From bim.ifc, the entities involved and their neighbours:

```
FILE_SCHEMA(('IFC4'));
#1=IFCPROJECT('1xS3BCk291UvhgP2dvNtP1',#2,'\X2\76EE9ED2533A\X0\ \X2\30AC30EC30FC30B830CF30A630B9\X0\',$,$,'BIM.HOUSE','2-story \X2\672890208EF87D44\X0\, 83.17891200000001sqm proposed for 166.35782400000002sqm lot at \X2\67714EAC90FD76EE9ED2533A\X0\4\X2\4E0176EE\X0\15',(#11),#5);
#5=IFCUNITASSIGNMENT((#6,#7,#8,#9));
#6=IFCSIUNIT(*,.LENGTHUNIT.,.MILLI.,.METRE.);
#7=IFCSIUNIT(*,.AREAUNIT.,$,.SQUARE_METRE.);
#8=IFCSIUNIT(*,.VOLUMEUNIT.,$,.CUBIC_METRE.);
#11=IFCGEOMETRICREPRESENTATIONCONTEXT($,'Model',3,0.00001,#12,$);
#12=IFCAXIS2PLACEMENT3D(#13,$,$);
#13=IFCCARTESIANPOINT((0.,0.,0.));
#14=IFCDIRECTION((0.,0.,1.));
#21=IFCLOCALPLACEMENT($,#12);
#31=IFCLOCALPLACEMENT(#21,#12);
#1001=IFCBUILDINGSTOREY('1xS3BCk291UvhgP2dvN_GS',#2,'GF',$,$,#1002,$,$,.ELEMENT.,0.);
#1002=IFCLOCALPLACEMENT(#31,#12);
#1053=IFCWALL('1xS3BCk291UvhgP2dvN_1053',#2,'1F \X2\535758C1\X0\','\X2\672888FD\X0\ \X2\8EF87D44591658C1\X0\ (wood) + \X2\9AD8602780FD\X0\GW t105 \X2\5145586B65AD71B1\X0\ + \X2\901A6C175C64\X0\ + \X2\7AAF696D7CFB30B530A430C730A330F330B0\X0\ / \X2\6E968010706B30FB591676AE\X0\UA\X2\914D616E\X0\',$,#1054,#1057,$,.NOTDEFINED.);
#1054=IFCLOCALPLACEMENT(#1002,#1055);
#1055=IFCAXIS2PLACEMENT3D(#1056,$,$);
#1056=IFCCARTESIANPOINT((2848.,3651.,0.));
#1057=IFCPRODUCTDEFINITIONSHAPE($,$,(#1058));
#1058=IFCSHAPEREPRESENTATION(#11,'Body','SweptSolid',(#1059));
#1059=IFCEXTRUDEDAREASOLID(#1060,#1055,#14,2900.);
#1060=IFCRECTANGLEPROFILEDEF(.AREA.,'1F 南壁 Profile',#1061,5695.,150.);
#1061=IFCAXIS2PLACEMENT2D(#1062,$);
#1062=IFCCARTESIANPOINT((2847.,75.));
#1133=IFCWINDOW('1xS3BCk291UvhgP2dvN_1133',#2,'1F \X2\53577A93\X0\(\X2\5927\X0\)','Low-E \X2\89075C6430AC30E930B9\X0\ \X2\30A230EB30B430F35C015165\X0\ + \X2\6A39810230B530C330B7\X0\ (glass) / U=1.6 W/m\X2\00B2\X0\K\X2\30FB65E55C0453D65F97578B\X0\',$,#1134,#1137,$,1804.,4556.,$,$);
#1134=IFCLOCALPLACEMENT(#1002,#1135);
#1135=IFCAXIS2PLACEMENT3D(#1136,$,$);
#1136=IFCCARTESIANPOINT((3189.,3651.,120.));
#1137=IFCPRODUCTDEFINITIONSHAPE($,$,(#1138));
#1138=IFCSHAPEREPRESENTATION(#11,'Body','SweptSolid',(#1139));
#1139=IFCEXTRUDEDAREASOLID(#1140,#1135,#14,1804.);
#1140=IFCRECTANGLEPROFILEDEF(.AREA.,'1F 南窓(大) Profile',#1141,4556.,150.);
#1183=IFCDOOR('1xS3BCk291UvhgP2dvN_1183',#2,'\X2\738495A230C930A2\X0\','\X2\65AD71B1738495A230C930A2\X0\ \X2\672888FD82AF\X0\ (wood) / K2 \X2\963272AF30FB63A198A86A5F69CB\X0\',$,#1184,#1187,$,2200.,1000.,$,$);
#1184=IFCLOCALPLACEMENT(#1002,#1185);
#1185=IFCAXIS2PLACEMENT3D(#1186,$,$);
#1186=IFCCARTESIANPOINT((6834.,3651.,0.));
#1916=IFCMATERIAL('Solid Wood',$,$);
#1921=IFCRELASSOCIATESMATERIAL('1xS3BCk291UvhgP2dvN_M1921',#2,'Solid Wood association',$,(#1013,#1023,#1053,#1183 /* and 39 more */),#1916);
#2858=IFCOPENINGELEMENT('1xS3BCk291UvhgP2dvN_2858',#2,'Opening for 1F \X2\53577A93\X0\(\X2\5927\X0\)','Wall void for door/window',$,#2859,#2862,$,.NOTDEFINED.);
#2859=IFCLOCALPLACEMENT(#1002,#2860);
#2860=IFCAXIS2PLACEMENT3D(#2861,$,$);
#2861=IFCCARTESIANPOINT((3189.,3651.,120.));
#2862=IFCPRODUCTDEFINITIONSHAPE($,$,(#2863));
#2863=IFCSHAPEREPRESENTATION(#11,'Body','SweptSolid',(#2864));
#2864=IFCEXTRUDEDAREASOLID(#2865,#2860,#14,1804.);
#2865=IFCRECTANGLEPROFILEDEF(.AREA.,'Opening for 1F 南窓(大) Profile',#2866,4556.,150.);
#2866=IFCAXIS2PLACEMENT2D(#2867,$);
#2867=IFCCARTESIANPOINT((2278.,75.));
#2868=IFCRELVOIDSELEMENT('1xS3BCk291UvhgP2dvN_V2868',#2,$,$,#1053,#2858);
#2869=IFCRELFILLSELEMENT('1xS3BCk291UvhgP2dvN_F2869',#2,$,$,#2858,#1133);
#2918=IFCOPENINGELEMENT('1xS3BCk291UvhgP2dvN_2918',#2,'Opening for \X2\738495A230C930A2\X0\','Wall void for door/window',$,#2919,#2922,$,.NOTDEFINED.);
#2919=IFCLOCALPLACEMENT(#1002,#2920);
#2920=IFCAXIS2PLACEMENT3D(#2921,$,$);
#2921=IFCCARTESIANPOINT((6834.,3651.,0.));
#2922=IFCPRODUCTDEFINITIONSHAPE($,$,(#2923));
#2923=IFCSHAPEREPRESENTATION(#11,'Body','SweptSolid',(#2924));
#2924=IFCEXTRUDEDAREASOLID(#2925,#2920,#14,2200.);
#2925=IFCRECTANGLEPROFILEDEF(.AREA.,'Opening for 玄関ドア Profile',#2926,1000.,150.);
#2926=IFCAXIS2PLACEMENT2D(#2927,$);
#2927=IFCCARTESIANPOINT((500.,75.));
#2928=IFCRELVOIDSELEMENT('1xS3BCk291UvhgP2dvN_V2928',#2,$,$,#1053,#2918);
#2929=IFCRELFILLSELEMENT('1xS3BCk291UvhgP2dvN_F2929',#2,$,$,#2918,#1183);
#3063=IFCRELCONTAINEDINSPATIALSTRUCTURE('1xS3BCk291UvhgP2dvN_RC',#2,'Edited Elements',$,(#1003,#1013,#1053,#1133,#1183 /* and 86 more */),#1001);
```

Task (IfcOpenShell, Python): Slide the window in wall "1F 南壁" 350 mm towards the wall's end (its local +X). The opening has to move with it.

```python
import ifcopenshell
import ifcopenshell.api.geometry
import ifcopenshell.util.placement

model = ifcopenshell.open("bim.ifc")

window = model.by_guid("1xS3BCk291UvhgP2dvN_1133")
opening = window.FillsVoids[0].RelatingOpeningElement
wall = opening.VoidsElements[0].RelatingBuildingElement

wall_matrix = ifcopenshell.util.placement.get_local_placement(wall.ObjectPlacement)
shift = wall_matrix[:3, 0] * 350.0
before = ifcopenshell.util.placement.get_local_placement(window.ObjectPlacement)[:3, 3].copy()

# The window is not placed relative to its opening, so move both.
for product in (opening, window):
    matrix = ifcopenshell.util.placement.get_local_placement(product.ObjectPlacement)
    matrix[:3, 3] += shift
    ifcopenshell.api.geometry.edit_object_placement(model, product=product, matrix=matrix, is_si=False)

after = ifcopenshell.util.placement.get_local_placement(window.ObjectPlacement)[:3, 3]
print("window moved by", (after - before).round(3) + 0.0)

model.write("bim_edited.ifc")
```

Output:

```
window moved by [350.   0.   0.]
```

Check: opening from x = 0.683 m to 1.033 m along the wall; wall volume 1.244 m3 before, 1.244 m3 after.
